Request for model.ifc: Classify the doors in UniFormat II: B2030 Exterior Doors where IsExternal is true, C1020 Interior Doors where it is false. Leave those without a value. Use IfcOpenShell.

First a look at what the model holds.

```python
import ifcopenshell
import ifcopenshell.util.element

model = ifcopenshell.open("model.ifc")
print(model.schema)
print("classifications:", [c.Name for c in model.by_type("IfcClassification")])
values = [ifcopenshell.util.element.get_pset(e, "Pset_DoorCommon", "IsExternal") for e in model.by_type("IfcDoor")]
for value in (True, False, None):
    print("IsExternal", value, values.count(value))
```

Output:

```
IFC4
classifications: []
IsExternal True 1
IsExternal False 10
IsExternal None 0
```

```python
import ifcopenshell
import ifcopenshell.api.classification
import ifcopenshell.util.element

model = ifcopenshell.open("model.ifc")

system = ifcopenshell.api.classification.add_classification(model, classification="UniFormat II")

doors = model.by_type("IfcDoor")
external = {e: ifcopenshell.util.element.get_pset(e, "Pset_DoorCommon", "IsExternal") for e in doors}
for flag, code, name in ((True, "B2030", "Exterior Doors"), (False, "C1020", "Interior Doors")):
    products = [e for e in doors if external[e] is flag]
    ifcopenshell.api.classification.add_reference(
        model, products=products, classification=system, identification=code, name=name
    )
    print(code, len(products))

model.write("model_rev.ifc")
```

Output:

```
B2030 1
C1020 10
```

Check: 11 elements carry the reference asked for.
